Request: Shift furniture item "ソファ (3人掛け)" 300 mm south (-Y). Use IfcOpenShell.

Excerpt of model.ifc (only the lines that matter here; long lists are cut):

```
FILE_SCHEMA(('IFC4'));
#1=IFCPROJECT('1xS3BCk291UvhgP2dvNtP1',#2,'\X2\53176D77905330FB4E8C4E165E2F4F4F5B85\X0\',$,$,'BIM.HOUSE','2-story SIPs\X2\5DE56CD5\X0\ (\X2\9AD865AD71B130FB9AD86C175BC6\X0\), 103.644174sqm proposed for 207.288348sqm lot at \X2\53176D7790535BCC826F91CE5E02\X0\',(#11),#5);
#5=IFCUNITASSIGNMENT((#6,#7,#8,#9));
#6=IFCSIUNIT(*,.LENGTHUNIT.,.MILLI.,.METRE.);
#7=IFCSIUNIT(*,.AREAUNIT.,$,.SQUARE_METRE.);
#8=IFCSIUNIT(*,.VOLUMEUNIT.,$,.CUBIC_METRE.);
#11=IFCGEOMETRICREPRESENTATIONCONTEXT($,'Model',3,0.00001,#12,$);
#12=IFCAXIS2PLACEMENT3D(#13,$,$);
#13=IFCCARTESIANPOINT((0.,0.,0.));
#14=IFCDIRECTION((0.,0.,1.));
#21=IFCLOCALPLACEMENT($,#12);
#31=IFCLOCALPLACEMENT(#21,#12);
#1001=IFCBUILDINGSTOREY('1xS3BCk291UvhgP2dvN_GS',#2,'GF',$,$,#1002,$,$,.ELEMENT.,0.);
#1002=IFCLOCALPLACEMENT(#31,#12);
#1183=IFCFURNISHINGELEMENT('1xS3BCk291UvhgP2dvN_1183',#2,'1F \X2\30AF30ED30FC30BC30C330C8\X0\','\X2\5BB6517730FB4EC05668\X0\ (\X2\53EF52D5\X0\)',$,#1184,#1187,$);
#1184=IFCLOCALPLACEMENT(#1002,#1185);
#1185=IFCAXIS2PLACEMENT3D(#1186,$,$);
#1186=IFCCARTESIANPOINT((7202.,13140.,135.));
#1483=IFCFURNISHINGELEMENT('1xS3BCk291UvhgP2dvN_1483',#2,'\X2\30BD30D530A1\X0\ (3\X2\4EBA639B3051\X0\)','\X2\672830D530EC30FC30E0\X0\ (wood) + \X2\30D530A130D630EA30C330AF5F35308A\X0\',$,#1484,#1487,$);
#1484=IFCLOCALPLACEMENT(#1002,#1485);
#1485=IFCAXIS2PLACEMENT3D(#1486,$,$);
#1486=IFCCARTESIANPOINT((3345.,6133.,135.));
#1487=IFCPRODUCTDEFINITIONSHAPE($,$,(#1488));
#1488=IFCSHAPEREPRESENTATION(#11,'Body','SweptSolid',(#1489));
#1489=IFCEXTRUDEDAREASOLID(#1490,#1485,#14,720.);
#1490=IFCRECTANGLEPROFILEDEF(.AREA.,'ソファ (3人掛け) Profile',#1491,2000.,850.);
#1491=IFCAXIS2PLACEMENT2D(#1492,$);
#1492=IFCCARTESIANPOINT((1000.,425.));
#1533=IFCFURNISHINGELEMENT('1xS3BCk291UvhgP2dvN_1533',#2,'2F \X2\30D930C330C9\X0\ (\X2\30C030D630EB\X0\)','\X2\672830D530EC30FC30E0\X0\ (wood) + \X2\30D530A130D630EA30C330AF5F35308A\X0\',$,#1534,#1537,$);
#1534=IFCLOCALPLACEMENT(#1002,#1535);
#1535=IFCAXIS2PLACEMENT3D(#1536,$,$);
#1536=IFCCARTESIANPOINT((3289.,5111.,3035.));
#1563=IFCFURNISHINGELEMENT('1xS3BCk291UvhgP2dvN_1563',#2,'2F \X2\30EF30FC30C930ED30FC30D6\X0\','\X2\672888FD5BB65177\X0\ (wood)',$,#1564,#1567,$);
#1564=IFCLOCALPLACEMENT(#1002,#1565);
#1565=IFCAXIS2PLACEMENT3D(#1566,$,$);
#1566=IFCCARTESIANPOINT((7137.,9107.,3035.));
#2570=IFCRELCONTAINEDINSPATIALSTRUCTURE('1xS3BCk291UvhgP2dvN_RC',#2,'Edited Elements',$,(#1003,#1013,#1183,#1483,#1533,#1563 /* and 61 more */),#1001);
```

```python
import ifcopenshell
import ifcopenshell.api.geometry
import ifcopenshell.util.placement

model = ifcopenshell.open("model.ifc")

item = model.by_guid("1xS3BCk291UvhgP2dvN_1483")
matrix = ifcopenshell.util.placement.get_local_placement(item.ObjectPlacement)
matrix[1, 3] -= 300.0
ifcopenshell.api.geometry.edit_object_placement(model, product=item, matrix=matrix, is_si=False)

print(ifcopenshell.util.placement.get_local_placement(item.ObjectPlacement).round(3) + 0.0)

model.write("model_edited.ifc")
```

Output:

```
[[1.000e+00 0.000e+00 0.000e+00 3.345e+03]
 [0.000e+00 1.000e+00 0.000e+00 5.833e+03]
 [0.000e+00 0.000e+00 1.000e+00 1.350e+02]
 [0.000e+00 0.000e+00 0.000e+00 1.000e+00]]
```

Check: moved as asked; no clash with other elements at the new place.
